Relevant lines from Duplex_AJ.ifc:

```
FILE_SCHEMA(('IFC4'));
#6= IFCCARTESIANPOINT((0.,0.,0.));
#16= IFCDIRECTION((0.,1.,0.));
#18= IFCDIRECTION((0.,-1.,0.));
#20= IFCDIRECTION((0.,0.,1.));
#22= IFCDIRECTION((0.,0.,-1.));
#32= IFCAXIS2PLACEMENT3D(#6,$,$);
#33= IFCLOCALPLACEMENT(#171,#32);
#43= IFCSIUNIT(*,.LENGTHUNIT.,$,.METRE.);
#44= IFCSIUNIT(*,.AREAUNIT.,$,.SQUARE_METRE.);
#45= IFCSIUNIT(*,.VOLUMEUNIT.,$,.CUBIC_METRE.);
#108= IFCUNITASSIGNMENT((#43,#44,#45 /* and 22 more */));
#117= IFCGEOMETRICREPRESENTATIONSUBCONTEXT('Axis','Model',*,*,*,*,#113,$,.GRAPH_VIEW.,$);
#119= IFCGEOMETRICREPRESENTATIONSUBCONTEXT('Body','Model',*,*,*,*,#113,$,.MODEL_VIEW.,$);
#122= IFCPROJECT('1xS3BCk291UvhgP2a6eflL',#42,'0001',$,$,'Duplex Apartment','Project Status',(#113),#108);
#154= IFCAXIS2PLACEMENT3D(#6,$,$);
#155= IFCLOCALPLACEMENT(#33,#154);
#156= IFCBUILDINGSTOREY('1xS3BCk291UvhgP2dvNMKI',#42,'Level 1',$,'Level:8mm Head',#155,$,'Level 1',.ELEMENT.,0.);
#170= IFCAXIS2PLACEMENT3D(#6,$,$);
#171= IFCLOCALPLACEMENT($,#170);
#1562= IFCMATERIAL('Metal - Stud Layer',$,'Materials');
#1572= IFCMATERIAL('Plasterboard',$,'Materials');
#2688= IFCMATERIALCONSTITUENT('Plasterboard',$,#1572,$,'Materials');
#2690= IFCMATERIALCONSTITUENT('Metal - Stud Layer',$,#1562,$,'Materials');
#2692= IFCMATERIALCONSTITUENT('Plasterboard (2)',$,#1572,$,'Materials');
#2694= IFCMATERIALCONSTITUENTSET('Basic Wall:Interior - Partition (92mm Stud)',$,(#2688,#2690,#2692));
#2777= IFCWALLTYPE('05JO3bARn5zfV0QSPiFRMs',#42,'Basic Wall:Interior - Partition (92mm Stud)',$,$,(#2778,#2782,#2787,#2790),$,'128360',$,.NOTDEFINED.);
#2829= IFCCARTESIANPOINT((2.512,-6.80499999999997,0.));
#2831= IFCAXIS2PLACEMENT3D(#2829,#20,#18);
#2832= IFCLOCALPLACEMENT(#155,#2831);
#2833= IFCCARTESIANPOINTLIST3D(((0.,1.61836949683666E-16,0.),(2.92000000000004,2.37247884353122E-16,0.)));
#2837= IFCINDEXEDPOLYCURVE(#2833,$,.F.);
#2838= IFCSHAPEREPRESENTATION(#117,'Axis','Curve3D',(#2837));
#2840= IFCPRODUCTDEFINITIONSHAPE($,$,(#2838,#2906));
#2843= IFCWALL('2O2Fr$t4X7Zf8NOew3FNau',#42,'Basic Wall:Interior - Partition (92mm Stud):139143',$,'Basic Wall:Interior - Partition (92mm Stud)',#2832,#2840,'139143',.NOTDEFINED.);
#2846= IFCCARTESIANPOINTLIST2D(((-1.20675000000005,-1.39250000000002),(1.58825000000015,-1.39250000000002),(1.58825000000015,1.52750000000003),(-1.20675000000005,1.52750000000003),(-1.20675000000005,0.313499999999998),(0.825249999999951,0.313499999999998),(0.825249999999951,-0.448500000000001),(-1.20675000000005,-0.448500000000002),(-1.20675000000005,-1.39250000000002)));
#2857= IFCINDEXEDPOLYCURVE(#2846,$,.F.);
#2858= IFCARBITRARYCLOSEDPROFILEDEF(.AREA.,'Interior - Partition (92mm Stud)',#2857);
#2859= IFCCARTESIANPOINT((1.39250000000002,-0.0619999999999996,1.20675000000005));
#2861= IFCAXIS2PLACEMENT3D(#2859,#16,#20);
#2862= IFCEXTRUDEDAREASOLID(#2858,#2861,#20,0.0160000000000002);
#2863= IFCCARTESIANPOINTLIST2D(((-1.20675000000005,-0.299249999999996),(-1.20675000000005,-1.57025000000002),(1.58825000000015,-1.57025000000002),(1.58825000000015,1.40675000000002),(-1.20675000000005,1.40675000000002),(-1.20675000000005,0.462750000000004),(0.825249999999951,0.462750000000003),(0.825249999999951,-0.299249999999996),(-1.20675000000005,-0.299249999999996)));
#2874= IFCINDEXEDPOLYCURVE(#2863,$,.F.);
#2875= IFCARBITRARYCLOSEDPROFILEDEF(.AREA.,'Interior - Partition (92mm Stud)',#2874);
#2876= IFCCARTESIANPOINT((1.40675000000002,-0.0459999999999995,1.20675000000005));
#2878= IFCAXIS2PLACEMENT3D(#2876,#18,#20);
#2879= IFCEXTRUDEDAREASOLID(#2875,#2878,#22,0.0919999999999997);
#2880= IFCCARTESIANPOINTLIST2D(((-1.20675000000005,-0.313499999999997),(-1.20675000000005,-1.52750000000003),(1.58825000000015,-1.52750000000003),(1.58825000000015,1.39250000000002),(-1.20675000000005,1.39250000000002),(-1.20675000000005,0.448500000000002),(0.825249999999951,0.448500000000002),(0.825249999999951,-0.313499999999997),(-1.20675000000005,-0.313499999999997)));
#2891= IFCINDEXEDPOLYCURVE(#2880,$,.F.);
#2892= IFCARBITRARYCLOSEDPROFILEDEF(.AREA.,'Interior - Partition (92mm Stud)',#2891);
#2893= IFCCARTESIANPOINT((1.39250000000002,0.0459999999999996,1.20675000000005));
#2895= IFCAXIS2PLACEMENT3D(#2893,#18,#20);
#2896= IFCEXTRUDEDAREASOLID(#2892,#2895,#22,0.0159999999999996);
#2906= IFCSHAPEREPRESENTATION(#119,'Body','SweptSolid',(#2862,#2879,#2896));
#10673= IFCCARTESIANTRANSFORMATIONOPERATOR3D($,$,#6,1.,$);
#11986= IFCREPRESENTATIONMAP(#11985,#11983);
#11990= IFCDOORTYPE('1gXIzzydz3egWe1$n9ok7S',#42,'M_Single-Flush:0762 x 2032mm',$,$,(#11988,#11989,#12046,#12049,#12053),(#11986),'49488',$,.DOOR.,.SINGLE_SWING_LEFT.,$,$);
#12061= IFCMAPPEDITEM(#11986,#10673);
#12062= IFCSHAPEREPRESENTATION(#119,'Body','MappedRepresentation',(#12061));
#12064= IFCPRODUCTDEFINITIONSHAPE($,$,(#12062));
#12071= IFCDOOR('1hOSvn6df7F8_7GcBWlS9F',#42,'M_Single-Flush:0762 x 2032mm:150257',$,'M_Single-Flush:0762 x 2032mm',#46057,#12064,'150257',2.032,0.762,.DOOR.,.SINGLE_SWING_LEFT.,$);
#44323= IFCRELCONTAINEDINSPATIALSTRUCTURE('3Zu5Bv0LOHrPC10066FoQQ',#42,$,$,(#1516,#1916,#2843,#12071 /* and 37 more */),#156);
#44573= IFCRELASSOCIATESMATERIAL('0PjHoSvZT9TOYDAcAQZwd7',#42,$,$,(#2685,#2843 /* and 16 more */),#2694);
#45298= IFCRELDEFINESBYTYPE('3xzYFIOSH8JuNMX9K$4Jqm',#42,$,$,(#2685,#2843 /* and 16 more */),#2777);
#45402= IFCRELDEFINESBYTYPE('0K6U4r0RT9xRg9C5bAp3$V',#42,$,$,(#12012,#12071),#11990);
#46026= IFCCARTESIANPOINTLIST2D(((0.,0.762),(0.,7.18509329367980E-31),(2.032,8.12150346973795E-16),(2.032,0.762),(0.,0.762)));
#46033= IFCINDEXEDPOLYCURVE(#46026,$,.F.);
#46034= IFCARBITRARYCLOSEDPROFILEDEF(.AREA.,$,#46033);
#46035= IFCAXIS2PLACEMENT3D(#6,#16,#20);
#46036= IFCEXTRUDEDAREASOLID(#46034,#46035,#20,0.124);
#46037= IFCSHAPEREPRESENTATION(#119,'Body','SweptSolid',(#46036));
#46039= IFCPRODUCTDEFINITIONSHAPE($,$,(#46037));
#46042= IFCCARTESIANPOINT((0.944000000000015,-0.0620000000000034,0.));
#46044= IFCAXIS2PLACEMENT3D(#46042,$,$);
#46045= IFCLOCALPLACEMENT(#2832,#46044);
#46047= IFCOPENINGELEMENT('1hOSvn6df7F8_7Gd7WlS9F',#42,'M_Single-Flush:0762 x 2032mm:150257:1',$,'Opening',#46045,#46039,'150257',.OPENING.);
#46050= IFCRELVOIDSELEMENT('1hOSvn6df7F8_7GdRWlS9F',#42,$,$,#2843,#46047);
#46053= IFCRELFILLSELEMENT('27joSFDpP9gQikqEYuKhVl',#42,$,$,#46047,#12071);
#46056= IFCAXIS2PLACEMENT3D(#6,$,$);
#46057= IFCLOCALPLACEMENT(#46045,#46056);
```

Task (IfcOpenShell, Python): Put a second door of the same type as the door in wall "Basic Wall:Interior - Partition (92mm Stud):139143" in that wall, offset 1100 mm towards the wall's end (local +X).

```python
import ifcopenshell
import ifcopenshell.api.feature
import ifcopenshell.api.geometry
import ifcopenshell.api.root
import ifcopenshell.geom
import ifcopenshell.util.element
import ifcopenshell.util.placement
import ifcopenshell.util.shape

model = ifcopenshell.open("Duplex_AJ.ifc")
settings = ifcopenshell.geom.settings()


def volume(element):
    """Net volume in cubic metres, openings subtracted."""
    shape = ifcopenshell.geom.create_shape(settings, element)
    return ifcopenshell.util.shape.get_volume(shape.geometry)


def reuse_history(source, copy):
    """copy_class also copies each property set's owner history, people and application; keep the originals."""
    for rel in copy.IsDefinedBy:
        if rel.is_a("IfcRelDefinesByProperties") and (history := rel.RelatingPropertyDefinition.OwnerHistory):
            rel.RelatingPropertyDefinition.OwnerHistory = source.OwnerHistory
            ifcopenshell.util.element.remove_deep2(model, history)


door = model.by_id(12071)
opening = door.FillsVoids[0].RelatingOpeningElement
wall = opening.VoidsElements[0].RelatingBuildingElement
before = volume(wall)
shift = ifcopenshell.util.placement.get_local_placement(wall.ObjectPlacement)[:3, 0] * 1.1

# copy_class copies the void relationship, type, container and properties, but no geometry.
new_opening = ifcopenshell.api.root.copy_class(model, product=opening)
new_opening.Representation = ifcopenshell.util.element.copy_deep(
    model, opening.Representation, exclude=["IfcGeometricRepresentationContext", "IfcRepresentationMap"]
)
new_opening.Name = "M_Single-Flush:0762 x 2032mm"
new_opening.Tag = None
new_door = ifcopenshell.api.root.copy_class(model, product=door)
new_door.Representation = ifcopenshell.util.element.copy_deep(
    model, door.Representation, exclude=["IfcGeometricRepresentationContext", "IfcRepresentationMap"]
)
new_door.Name = "M_Single-Flush:0762 x 2032mm"
new_door.Tag = None
reuse_history(door, new_door)
ifcopenshell.api.feature.add_filling(model, opening=new_opening, element=new_door)

for old, new in ((opening, new_opening), (door, new_door)):
    matrix = ifcopenshell.util.placement.get_local_placement(old.ObjectPlacement)
    matrix[:3, 3] += shift
    ifcopenshell.api.geometry.edit_object_placement(model, product=new, matrix=matrix, is_si=False)

after = volume(wall)

print(f"wall volume {before:.3f} -> {after:.3f} m3")

model.write("Duplex_AJ_edited.ifc")
```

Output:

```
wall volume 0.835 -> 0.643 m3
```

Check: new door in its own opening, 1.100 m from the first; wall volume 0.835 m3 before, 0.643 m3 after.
